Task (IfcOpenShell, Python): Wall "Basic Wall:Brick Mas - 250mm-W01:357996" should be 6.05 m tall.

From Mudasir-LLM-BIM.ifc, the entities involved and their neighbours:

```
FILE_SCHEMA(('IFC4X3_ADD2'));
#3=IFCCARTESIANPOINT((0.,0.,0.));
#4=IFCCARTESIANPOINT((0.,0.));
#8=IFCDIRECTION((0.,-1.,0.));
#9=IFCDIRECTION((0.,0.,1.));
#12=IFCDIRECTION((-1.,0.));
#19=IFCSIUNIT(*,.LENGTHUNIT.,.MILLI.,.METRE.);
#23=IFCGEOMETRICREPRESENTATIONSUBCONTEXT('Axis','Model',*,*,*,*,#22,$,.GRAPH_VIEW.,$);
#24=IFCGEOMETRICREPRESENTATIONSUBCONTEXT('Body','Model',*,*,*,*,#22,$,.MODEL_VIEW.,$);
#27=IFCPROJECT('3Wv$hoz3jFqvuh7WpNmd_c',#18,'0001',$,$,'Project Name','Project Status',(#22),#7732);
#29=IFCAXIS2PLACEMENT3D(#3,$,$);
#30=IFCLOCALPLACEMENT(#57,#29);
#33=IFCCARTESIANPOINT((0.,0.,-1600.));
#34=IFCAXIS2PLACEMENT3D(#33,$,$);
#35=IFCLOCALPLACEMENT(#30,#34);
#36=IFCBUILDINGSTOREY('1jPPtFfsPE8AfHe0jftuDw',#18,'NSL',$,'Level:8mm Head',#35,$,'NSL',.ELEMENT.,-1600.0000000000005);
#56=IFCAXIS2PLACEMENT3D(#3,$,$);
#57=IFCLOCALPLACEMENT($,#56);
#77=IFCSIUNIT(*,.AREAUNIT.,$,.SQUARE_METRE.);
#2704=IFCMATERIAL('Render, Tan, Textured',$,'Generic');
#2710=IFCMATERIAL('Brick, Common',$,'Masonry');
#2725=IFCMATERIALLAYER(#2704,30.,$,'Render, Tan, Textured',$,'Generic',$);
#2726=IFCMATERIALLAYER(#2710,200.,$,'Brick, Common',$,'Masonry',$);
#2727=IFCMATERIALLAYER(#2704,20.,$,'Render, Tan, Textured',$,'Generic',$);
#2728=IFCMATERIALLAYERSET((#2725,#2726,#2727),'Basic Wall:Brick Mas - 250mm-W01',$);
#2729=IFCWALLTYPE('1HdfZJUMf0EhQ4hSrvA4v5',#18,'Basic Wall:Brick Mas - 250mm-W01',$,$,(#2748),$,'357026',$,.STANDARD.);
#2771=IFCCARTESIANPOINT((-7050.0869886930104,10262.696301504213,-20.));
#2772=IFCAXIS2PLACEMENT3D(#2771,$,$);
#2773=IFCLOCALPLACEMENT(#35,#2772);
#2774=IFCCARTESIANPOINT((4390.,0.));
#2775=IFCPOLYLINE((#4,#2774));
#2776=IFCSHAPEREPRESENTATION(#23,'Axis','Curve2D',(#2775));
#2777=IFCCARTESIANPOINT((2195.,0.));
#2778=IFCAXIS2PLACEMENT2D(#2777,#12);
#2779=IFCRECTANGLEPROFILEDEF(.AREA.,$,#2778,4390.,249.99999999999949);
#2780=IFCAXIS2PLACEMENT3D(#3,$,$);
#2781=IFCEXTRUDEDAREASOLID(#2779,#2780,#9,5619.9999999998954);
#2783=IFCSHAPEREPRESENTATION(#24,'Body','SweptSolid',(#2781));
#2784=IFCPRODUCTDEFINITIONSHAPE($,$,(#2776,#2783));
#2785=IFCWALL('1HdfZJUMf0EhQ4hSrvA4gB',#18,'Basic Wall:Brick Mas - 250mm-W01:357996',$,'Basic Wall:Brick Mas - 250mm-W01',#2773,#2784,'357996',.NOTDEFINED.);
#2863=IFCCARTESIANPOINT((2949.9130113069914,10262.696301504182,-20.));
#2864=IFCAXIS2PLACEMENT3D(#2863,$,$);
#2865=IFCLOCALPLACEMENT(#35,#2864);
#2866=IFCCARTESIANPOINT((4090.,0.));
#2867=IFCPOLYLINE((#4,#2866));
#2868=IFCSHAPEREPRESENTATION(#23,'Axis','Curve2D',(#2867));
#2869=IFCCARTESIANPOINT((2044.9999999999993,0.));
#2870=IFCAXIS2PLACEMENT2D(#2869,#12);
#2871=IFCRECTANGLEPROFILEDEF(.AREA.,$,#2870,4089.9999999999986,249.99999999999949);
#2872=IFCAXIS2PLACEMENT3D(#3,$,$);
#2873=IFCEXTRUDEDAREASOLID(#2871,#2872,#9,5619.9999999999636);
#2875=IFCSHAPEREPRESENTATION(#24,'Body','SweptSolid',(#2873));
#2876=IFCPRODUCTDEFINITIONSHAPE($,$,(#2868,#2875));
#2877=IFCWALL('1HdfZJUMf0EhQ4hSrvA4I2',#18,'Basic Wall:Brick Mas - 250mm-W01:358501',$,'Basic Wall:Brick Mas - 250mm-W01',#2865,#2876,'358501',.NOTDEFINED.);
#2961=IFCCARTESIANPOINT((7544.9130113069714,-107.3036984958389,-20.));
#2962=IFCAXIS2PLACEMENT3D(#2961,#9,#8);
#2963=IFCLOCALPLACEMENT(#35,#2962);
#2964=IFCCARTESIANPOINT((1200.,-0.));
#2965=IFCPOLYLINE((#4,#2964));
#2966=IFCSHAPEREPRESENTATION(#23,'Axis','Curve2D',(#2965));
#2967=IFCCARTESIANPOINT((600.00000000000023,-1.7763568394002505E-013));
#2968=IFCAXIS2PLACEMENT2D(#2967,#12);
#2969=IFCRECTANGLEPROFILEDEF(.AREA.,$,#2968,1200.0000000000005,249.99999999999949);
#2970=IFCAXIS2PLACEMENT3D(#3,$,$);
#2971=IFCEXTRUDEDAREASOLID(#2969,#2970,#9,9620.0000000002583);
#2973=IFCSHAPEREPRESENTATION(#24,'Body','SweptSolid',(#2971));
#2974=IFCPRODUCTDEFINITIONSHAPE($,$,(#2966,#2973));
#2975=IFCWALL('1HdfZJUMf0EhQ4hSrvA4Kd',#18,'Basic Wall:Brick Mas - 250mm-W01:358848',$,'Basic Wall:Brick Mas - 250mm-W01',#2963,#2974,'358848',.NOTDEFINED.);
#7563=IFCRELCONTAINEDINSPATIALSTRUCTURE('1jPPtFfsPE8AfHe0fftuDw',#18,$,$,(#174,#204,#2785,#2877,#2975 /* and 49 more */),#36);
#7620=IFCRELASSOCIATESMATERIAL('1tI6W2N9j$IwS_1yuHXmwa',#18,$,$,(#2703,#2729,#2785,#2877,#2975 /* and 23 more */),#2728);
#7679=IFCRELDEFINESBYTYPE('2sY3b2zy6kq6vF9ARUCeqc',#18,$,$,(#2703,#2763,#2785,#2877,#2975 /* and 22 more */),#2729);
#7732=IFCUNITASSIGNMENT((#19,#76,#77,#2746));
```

```python
import ifcopenshell
import ifcopenshell.geom
import ifcopenshell.util.representation
import ifcopenshell.util.shape
import ifcopenshell.util.unit

model = ifcopenshell.open("Mudasir-LLM-BIM.ifc")
unit_scale = ifcopenshell.util.unit.calculate_unit_scale(model)
settings = ifcopenshell.geom.settings()


def volume(element):
    """Net volume in cubic metres, openings subtracted."""
    shape = ifcopenshell.geom.create_shape(settings, element)
    return ifcopenshell.util.shape.get_volume(shape.geometry)


wall = model.by_guid("1HdfZJUMf0EhQ4hSrvA4gB")
before = volume(wall)

body = ifcopenshell.util.representation.get_representation(wall, "Model", "Body")
solid = body.Items[0]
old_height = solid.Depth
solid.Depth = 6.05 / unit_scale
after = volume(wall)

print(f"height {old_height:g} -> {solid.Depth:g}, volume {before:.3f} -> {after:.3f} m3")

model.write("Mudasir-LLM-BIM_updated.ifc")
```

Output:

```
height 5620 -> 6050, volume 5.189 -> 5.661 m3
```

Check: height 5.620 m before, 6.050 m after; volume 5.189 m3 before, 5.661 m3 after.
